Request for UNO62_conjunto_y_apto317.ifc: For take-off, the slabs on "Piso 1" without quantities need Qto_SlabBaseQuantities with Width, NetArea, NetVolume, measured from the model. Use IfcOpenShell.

First a look at what the model holds.

```python
import ifcopenshell
import ifcopenshell.util.element
import ifcopenshell.util.unit

model = ifcopenshell.open("UNO62_conjunto_y_apto317.ifc")
print(model.schema)
for unit_type in ("LENGTHUNIT", "AREAUNIT", "VOLUMEUNIT"):
    print(unit_type, ifcopenshell.util.unit.calculate_unit_scale(model, unit_type))
storey = next(s for s in model.by_type("IfcBuildingStorey") if s.Name == "Piso 1")
slabs = [e for e in ifcopenshell.util.element.get_decomposition(storey) if e.is_a("IfcSlab")]
for e in sorted(slabs, key=lambda e: e.id()):
    print(e.id(), e.is_a(), e.Name, list(ifcopenshell.util.element.get_psets(e, qtos_only=True)), sep=" | ")
```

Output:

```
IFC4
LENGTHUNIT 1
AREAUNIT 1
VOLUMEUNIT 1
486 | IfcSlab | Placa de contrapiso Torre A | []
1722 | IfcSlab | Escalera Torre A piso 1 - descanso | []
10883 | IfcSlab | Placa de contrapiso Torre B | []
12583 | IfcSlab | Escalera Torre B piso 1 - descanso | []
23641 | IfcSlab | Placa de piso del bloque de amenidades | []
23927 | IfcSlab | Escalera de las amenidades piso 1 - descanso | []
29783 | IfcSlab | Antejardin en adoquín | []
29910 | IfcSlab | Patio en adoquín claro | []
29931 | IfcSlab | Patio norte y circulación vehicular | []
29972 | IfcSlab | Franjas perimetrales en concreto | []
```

```python
import ifcopenshell
import ifcopenshell.api.pset
import ifcopenshell.geom
import ifcopenshell.util.element
import ifcopenshell.util.shape
import ifcopenshell.util.unit

model = ifcopenshell.open("UNO62_conjunto_y_apto317.ifc")
unit_scale = ifcopenshell.util.unit.calculate_unit_scale(model)
area_scale = ifcopenshell.util.unit.calculate_unit_scale(model, "AREAUNIT")
volume_scale = ifcopenshell.util.unit.calculate_unit_scale(model, "VOLUMEUNIT")
settings = ifcopenshell.geom.settings()

storey = next(s for s in model.by_type("IfcBuildingStorey") if s.Name == "Piso 1")
slabs = [e for e in ifcopenshell.util.element.get_decomposition(storey) if e.is_a("IfcSlab")]

for e in sorted(slabs, key=lambda e: e.id()):
    if ifcopenshell.util.element.get_psets(e, qtos_only=True, should_inherit=False):
        continue
    # Geometry comes back in metres, in the element's own axes.
    shape = ifcopenshell.geom.create_shape(settings, e)
    values = {
        "Width": ifcopenshell.util.shape.get_z(shape.geometry) / unit_scale,
        "NetArea": ifcopenshell.util.shape.get_footprint_area(shape.geometry) / area_scale,
        "NetVolume": ifcopenshell.util.shape.get_volume(shape.geometry) / volume_scale,
    }
    qto = ifcopenshell.api.pset.add_qto(model, product=e, name="Qto_SlabBaseQuantities")
    ifcopenshell.api.pset.edit_qto(model, qto=qto, properties=values)
    print(e.id(), {k: round(v, 3) for k, v in values.items()})

model.write("UNO62_conjunto_y_apto317_edited.ifc")
```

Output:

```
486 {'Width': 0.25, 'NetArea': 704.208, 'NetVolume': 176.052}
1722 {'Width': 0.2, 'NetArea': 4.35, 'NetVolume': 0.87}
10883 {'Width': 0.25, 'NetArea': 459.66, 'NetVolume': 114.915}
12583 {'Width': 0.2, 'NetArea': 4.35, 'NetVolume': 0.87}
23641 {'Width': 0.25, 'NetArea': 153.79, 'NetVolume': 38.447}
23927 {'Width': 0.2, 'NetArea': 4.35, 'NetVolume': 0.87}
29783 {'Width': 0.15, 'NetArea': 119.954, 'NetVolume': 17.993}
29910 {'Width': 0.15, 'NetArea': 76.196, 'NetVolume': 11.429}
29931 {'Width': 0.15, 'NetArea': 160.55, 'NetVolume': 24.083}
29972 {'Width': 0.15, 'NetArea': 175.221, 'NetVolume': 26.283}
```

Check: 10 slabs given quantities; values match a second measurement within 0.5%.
